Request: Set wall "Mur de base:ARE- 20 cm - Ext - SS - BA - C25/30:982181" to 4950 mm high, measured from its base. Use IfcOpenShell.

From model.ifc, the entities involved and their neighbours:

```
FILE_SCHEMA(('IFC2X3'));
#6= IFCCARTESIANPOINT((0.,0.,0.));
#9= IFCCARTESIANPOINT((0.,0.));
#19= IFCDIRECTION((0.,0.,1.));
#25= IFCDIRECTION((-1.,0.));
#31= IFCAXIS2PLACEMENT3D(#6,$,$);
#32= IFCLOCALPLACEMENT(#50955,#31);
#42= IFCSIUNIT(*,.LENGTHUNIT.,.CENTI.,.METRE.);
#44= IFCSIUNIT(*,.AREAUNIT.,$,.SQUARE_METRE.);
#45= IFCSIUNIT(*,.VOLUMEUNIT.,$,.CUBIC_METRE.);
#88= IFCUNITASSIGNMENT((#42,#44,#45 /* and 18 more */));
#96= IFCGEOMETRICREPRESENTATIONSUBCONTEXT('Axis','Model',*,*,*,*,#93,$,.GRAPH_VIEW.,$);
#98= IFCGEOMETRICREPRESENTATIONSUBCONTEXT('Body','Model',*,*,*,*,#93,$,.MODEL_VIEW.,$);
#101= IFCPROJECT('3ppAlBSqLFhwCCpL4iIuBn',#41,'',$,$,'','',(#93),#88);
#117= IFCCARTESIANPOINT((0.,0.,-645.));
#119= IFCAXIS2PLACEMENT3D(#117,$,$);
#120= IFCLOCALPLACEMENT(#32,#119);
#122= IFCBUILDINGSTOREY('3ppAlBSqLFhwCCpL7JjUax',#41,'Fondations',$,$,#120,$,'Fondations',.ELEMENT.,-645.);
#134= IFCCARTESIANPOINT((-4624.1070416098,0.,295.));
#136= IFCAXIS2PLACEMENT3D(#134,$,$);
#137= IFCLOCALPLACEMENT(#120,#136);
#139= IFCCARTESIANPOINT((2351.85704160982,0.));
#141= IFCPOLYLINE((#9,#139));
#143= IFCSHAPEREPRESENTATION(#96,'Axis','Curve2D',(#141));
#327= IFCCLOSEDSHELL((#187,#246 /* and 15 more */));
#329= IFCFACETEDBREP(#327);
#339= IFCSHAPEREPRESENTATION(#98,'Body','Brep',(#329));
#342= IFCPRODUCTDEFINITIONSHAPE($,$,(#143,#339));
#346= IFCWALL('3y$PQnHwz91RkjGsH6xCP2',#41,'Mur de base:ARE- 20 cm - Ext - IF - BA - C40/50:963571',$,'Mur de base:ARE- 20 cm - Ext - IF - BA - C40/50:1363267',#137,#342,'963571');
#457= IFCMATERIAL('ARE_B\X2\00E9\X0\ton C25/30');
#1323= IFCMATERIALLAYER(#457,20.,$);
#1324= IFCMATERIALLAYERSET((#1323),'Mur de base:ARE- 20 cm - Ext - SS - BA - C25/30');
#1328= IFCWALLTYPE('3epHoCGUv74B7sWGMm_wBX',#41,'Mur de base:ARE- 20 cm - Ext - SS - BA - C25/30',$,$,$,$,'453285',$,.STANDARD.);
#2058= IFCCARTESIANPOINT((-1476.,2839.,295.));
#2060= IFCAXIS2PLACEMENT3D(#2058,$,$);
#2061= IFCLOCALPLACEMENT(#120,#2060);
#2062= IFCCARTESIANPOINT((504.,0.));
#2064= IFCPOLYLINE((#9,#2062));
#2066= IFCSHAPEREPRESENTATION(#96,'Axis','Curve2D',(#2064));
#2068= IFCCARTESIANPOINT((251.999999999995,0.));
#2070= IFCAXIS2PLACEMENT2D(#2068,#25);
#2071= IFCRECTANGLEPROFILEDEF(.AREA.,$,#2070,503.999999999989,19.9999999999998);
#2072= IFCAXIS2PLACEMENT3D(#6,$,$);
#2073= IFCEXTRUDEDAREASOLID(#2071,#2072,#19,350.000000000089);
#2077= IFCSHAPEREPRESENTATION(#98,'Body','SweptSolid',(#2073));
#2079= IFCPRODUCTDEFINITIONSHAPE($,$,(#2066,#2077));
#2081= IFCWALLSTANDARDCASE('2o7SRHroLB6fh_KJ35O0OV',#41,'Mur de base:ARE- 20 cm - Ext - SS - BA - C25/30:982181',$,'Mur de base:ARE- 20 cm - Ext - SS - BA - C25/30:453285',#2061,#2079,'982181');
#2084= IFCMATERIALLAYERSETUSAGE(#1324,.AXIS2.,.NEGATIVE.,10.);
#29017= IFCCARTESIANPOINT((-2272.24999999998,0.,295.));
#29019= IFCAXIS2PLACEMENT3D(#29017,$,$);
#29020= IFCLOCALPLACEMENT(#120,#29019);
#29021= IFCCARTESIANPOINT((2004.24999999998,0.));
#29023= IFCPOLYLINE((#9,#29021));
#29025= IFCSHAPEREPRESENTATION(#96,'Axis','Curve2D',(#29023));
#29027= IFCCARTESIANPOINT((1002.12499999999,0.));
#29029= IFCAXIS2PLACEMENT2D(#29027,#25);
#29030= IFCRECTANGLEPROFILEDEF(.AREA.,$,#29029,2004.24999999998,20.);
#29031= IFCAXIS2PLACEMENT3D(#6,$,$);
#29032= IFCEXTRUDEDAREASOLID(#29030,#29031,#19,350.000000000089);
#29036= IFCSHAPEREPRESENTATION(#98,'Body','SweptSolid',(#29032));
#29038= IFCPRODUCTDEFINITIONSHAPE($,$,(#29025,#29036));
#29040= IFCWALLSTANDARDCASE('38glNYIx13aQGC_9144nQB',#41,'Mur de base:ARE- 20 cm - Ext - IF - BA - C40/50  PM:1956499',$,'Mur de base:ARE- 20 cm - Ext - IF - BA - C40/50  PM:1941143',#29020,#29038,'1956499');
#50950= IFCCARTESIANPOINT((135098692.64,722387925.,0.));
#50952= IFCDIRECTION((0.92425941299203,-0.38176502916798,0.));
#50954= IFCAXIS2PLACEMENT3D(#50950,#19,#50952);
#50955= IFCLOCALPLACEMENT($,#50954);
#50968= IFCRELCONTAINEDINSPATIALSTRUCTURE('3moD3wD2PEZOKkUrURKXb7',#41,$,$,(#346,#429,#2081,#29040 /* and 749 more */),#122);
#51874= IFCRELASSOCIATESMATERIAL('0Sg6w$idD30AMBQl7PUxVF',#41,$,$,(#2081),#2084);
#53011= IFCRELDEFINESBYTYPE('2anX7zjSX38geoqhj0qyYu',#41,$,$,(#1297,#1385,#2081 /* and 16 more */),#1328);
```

```python
import ifcopenshell
import ifcopenshell.geom
import ifcopenshell.util.representation
import ifcopenshell.util.shape
import ifcopenshell.util.unit

model = ifcopenshell.open("model.ifc")
unit_scale = ifcopenshell.util.unit.calculate_unit_scale(model)
settings = ifcopenshell.geom.settings()


def volume(element):
    """Net volume in cubic metres, openings subtracted."""
    shape = ifcopenshell.geom.create_shape(settings, element)
    return ifcopenshell.util.shape.get_volume(shape.geometry)


wall = model.by_id(2081)
before = volume(wall)

body = ifcopenshell.util.representation.get_representation(wall, "Model", "Body")
solid = body.Items[0]
old_height = solid.Depth
solid.Depth = 4.95 / unit_scale
after = volume(wall)

print(f"height {old_height:g} -> {solid.Depth:g}, volume {before:.3f} -> {after:.3f} m3")

model.write("model_edited.ifc")
```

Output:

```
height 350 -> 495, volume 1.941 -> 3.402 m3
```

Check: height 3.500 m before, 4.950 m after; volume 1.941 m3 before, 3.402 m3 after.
